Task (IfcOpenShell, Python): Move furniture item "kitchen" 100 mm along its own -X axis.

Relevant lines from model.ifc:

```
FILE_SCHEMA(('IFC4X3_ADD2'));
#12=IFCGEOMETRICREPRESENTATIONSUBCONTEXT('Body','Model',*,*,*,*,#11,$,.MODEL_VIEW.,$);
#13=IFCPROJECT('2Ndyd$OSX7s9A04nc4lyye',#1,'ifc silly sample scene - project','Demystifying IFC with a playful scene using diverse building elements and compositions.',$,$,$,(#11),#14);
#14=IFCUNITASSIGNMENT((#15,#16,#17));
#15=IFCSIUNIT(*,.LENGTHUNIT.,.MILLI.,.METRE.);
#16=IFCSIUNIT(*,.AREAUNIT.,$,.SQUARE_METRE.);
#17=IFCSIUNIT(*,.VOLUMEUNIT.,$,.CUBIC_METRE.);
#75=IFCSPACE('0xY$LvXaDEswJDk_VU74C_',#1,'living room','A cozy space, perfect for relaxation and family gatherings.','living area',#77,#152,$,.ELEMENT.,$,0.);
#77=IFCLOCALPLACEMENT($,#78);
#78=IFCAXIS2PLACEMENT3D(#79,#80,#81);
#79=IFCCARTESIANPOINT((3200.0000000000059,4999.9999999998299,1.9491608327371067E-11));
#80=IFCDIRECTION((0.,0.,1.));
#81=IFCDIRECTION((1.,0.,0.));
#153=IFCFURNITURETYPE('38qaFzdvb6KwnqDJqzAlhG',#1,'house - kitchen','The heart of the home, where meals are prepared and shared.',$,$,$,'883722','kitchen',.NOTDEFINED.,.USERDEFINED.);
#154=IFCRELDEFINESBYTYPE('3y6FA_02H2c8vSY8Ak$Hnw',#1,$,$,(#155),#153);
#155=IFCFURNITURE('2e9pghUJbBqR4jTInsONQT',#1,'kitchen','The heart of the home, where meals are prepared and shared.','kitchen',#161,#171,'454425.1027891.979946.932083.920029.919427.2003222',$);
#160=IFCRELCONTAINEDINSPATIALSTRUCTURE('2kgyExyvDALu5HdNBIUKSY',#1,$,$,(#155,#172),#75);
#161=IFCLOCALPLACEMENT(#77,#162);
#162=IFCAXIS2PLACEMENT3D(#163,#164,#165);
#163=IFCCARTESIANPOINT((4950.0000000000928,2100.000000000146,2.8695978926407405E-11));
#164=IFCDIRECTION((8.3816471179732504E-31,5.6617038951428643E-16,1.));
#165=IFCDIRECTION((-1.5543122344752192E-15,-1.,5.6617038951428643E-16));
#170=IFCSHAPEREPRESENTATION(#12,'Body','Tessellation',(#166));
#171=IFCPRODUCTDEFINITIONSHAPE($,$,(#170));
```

```python
import ifcopenshell
import ifcopenshell.api.geometry
import ifcopenshell.util.placement

model = ifcopenshell.open("model.ifc")

item = model.by_guid("2e9pghUJbBqR4jTInsONQT")
matrix = ifcopenshell.util.placement.get_local_placement(item.ObjectPlacement)
matrix[:3, 3] -= matrix[:3, 0] * 100.0
ifcopenshell.api.geometry.edit_object_placement(model, product=item, matrix=matrix, is_si=False)

print(ifcopenshell.util.placement.get_local_placement(item.ObjectPlacement).round(3) + 0.0)

model.write("model_rev.ifc")
```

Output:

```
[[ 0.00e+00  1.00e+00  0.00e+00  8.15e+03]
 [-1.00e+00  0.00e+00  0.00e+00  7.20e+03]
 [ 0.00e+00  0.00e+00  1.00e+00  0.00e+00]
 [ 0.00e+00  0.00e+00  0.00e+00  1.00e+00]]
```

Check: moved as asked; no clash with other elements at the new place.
